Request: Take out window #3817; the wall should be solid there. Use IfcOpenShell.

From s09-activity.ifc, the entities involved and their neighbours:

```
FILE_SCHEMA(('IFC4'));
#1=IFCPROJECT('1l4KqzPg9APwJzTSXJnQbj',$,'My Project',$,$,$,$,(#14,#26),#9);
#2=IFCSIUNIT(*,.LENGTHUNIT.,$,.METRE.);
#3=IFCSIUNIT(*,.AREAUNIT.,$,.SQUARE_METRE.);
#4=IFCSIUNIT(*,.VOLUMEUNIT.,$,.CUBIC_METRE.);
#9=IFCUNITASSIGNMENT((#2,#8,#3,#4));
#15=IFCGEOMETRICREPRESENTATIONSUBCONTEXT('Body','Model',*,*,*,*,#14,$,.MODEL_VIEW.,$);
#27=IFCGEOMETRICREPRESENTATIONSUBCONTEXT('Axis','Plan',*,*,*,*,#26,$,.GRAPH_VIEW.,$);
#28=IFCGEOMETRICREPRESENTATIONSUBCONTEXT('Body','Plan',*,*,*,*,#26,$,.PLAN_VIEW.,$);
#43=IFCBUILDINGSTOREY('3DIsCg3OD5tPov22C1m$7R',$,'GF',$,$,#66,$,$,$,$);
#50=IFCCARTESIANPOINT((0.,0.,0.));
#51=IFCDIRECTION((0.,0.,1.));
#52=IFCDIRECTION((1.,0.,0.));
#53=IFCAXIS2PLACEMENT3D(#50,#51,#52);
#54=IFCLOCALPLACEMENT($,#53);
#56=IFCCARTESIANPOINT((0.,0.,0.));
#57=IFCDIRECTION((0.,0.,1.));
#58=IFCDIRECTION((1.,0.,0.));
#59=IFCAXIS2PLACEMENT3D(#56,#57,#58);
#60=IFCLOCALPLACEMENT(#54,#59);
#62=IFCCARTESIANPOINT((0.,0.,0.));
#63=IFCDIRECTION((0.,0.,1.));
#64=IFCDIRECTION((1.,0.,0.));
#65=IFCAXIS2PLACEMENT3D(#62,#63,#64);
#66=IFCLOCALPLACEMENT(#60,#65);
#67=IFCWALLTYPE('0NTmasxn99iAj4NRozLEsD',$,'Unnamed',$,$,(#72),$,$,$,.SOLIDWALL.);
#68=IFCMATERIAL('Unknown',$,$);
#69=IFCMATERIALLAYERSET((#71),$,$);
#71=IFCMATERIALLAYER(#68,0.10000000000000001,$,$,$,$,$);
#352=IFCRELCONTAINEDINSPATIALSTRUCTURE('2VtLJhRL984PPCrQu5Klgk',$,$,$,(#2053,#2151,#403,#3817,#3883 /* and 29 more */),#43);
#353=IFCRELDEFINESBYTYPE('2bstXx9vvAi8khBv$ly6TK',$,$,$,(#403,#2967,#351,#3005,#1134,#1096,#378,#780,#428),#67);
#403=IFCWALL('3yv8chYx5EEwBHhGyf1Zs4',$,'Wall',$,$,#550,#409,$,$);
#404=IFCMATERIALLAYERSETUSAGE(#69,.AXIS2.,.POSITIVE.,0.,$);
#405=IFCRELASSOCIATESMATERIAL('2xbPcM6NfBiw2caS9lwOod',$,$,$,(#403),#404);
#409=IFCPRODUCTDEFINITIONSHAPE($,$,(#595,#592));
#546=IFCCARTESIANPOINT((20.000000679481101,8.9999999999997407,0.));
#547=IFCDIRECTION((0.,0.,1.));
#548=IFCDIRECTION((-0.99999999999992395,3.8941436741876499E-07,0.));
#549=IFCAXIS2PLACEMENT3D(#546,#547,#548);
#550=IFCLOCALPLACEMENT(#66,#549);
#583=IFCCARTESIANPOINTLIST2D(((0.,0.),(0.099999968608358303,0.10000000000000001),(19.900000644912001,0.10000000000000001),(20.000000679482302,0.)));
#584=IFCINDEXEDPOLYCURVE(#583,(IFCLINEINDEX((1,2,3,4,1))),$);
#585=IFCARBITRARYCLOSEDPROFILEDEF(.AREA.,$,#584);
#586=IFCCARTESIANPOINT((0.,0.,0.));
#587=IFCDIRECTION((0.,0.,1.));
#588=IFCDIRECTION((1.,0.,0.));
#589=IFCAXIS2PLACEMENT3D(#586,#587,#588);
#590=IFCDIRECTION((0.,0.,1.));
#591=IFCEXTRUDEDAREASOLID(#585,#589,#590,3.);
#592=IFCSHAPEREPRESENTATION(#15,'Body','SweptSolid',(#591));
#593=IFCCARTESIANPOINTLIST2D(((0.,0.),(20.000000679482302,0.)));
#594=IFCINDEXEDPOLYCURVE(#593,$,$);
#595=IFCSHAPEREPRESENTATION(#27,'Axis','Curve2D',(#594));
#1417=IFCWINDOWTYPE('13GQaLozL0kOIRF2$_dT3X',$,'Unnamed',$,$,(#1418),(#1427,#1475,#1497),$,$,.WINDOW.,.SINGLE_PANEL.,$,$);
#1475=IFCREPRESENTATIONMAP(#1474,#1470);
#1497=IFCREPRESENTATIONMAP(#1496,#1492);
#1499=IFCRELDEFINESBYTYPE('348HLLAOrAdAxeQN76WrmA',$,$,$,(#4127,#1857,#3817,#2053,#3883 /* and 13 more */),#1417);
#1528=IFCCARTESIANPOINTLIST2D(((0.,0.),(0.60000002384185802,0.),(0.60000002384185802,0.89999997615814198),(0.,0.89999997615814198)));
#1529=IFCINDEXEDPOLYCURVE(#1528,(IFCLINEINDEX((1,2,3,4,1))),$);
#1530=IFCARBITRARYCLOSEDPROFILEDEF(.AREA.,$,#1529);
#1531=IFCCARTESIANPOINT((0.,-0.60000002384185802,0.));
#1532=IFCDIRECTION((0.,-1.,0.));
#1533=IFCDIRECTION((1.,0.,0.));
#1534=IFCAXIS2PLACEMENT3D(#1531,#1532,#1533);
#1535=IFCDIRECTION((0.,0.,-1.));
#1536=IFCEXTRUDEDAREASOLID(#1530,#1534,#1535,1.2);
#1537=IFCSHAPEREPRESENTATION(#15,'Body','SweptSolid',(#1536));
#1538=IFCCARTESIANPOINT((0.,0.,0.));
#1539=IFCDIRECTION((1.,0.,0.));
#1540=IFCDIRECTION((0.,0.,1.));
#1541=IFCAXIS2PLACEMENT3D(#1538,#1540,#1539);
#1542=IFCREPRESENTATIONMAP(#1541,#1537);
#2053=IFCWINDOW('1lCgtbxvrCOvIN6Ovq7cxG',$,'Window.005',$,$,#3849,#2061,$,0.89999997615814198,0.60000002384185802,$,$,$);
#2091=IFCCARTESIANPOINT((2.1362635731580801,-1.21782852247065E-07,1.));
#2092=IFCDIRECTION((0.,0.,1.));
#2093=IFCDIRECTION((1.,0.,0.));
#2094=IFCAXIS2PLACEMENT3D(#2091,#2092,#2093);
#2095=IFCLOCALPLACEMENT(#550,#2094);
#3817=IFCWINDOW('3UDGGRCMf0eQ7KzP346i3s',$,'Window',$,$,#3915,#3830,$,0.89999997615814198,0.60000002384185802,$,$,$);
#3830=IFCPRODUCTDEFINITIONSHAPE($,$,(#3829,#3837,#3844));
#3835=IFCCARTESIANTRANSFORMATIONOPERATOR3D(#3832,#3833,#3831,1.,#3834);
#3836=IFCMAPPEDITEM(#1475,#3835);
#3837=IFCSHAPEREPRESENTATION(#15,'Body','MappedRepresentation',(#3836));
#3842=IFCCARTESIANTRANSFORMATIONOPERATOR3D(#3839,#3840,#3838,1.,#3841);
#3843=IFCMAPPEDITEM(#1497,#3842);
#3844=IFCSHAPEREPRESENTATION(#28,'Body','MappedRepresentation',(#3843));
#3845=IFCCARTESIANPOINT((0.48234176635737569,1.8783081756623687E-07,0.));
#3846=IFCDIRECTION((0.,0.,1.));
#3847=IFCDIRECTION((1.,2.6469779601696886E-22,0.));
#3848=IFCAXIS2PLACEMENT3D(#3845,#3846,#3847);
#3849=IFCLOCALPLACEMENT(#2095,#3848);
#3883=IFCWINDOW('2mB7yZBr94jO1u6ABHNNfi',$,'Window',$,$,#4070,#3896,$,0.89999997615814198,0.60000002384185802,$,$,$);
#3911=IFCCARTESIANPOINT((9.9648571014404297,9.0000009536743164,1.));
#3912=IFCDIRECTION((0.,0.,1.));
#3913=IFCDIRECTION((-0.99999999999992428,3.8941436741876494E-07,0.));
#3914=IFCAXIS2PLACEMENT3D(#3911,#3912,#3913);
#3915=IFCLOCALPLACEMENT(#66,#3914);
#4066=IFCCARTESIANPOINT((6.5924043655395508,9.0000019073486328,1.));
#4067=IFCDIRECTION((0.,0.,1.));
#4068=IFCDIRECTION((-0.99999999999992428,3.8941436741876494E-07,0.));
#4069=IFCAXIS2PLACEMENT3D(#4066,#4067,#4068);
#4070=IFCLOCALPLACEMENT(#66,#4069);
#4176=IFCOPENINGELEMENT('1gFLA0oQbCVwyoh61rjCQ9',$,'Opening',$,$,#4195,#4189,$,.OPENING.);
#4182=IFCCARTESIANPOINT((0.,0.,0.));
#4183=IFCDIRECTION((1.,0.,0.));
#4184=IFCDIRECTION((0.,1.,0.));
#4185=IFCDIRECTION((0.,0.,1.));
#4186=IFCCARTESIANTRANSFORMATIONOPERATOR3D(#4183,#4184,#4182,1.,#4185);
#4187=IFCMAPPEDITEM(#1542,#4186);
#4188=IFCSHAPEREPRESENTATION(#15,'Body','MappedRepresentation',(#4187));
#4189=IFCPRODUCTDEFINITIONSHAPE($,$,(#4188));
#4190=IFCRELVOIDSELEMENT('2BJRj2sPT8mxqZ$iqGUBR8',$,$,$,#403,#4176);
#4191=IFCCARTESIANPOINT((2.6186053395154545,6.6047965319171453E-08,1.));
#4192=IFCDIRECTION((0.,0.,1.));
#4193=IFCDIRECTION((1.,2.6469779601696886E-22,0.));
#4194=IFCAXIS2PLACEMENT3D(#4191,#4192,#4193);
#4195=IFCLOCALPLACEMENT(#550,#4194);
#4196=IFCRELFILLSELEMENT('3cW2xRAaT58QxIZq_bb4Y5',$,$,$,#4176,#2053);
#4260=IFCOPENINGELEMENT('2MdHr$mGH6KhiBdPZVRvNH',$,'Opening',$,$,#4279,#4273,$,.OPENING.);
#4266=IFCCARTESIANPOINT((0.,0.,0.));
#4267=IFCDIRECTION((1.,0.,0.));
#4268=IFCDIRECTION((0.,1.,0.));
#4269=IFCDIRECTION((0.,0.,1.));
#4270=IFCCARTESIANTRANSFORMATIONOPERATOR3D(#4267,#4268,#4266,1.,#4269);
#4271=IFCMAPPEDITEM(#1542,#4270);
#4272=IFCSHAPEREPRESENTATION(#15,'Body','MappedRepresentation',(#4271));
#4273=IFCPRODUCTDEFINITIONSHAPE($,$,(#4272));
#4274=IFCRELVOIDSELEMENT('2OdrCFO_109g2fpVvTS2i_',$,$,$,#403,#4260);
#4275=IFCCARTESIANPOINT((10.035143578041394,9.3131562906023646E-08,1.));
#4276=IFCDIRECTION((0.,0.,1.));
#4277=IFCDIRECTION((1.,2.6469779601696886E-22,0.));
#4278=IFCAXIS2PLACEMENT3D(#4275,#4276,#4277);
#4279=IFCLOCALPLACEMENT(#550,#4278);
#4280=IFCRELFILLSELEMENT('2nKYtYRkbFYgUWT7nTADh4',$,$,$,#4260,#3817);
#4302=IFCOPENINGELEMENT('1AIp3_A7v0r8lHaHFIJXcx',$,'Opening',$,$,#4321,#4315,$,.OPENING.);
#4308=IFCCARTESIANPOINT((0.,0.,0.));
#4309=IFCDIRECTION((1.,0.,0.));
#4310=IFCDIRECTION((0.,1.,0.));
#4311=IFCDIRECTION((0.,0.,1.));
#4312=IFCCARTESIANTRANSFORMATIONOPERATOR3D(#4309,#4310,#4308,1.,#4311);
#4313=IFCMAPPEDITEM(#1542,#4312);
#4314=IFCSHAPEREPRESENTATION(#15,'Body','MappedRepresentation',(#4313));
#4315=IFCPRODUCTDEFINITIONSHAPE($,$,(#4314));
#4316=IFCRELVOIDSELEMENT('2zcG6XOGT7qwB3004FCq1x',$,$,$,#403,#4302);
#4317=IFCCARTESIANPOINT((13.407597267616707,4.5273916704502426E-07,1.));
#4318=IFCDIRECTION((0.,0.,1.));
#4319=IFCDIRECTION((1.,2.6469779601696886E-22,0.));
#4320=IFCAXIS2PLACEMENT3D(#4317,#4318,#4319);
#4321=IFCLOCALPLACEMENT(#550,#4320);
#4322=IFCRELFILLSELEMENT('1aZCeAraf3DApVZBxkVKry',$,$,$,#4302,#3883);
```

```python
import ifcopenshell
import ifcopenshell.api.feature
import ifcopenshell.api.root
import ifcopenshell.geom
import ifcopenshell.util.shape

model = ifcopenshell.open("s09-activity.ifc")
settings = ifcopenshell.geom.settings()


def volume(element):
    """Net volume in cubic metres, openings subtracted."""
    shape = ifcopenshell.geom.create_shape(settings, element)
    return ifcopenshell.util.shape.get_volume(shape.geometry)


window = model.by_guid("3UDGGRCMf0eQ7KzP346i3s")
opening = window.FillsVoids[0].RelatingOpeningElement
wall = opening.VoidsElements[0].RelatingBuildingElement
before = volume(wall)

ifcopenshell.api.root.remove_product(model, product=window)
ifcopenshell.api.feature.remove_feature(model, feature=opening)

after = volume(wall)

print(f"wall volume {before:.3f} -> {after:.3f} m3")

model.write("s09-activity-out.ifc")
```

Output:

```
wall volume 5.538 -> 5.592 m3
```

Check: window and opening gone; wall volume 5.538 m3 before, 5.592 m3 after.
